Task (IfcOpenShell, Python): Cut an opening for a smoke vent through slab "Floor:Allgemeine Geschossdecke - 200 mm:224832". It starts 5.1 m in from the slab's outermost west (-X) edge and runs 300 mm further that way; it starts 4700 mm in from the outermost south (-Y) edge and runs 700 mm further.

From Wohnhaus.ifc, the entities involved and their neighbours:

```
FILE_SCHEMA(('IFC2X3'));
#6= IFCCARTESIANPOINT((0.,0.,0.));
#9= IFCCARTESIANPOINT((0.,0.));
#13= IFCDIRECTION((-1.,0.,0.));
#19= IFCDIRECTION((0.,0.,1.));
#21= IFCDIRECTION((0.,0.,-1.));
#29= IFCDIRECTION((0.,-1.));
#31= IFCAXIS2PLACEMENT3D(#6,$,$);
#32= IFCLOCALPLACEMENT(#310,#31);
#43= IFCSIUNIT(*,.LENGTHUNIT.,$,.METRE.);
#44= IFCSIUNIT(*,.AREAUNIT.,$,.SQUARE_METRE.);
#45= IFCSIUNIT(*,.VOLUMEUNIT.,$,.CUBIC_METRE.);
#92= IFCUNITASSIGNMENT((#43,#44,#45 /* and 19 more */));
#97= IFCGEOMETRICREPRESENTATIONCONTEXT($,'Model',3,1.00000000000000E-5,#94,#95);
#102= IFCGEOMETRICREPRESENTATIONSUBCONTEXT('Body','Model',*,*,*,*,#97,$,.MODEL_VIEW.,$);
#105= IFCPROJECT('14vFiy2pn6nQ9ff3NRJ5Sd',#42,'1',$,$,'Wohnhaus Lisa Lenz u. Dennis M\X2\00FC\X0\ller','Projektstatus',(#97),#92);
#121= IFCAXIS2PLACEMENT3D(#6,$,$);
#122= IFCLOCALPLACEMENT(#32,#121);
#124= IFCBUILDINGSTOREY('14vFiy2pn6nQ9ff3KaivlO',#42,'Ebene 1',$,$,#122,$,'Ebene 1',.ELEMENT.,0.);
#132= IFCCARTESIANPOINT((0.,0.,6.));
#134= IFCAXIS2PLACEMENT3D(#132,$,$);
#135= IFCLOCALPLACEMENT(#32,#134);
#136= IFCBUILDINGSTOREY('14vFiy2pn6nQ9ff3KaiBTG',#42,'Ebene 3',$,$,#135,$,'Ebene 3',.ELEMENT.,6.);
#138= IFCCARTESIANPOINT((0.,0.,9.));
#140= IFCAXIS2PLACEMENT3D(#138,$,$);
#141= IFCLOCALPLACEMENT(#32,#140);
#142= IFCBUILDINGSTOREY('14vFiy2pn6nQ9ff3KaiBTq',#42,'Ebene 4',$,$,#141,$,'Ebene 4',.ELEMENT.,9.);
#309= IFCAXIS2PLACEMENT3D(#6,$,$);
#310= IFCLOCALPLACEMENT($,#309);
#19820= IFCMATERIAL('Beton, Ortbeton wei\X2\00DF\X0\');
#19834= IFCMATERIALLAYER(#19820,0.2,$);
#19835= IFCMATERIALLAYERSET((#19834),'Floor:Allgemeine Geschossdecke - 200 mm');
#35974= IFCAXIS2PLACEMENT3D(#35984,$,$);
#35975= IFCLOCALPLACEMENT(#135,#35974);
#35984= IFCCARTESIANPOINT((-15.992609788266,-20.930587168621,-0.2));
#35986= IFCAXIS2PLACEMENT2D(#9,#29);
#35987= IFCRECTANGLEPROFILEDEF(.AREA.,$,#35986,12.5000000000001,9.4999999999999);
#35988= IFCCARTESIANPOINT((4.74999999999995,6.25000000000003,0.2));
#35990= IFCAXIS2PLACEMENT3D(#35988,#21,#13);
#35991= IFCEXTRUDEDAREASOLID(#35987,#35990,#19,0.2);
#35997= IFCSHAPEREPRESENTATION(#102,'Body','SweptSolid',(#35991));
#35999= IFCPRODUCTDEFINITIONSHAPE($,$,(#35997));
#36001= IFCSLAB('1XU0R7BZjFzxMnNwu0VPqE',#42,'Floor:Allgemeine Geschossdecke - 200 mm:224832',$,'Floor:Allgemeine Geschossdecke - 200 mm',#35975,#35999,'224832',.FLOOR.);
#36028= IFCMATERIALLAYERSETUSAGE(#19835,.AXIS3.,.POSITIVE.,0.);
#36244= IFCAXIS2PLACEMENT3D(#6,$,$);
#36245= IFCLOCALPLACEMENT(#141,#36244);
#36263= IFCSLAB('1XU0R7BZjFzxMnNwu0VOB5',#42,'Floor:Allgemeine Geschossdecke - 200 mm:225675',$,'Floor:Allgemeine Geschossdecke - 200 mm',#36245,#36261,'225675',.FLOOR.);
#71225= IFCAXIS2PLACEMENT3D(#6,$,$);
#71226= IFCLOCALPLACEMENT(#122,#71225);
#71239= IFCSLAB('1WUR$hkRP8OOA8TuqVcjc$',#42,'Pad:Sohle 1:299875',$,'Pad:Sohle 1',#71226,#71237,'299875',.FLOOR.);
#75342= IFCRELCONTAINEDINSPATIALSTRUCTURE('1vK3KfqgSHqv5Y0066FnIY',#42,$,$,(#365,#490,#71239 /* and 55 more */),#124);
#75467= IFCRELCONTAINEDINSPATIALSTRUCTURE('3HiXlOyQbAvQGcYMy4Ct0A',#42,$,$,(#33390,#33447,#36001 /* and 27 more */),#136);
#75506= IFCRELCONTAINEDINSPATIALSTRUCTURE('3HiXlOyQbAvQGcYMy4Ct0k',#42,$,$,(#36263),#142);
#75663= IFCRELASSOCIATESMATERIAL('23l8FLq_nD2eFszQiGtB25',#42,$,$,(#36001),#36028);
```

```python
import numpy as np
import ifcopenshell
import ifcopenshell.api.feature
import ifcopenshell.api.geometry
import ifcopenshell.api.root
import ifcopenshell.geom
import ifcopenshell.util.placement
import ifcopenshell.util.representation
import ifcopenshell.util.shape
import ifcopenshell.util.unit

model = ifcopenshell.open("Wohnhaus.ifc")
unit_scale = ifcopenshell.util.unit.calculate_unit_scale(model)
settings = ifcopenshell.geom.settings()


def volume(element):
    """Net volume in cubic metres, openings subtracted."""
    shape = ifcopenshell.geom.create_shape(settings, element)
    return ifcopenshell.util.shape.get_volume(shape.geometry)


slab = model.by_guid("1XU0R7BZjFzxMnNwu0VPqE")
before = volume(slab)

# Extent in the slab's own axes, in metres. The edges named are its -X and -Y sides.
slab_shape = ifcopenshell.geom.create_shape(settings, slab)
vertices = ifcopenshell.util.shape.get_vertices(slab_shape.geometry)
x_min, y_min, bottom = vertices.min(axis=0)
top = vertices[:, 2].max()

opening = ifcopenshell.api.root.create_entity(model, ifc_class="IfcOpeningElement", name="Smoke vent opening")
context = ifcopenshell.util.representation.get_context(model, "Model", "Body", "MODEL_VIEW")
width, depth = 0.3, 0.7
outline = [(0.0, 0.0), (width, 0.0), (width, depth), (0.0, depth), (0.0, 0.0)]
# Overshoot both faces by 50 mm so the cut is clean.
shape = ifcopenshell.api.geometry.add_slab_representation(
    model, context=context, depth=top - bottom + 0.1, polyline=outline
)
ifcopenshell.api.geometry.assign_representation(model, product=opening, representation=shape)

matrix = ifcopenshell.util.placement.get_local_placement(slab.ObjectPlacement)
matrix[:, 3] = matrix @ np.append(np.array([x_min + 5.1, y_min + 4.7, bottom - 0.05]) / unit_scale, 1.0)
ifcopenshell.api.geometry.edit_object_placement(model, product=opening, matrix=matrix, is_si=False)
ifcopenshell.api.feature.add_feature(model, feature=opening, element=slab)

after = volume(slab)

print(f"slab volume {before:.3f} -> {after:.3f} m3")

model.write("Wohnhaus_updated.ifc")
```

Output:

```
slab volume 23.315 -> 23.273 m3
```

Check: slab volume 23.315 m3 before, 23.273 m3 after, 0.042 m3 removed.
